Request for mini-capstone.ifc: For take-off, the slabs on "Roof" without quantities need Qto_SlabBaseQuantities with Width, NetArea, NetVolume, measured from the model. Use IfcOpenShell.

First a look at what the model holds.

```python
import ifcopenshell
import ifcopenshell.util.element
import ifcopenshell.util.unit

model = ifcopenshell.open("mini-capstone.ifc")
print(model.schema)
for unit_type in ("LENGTHUNIT", "AREAUNIT", "VOLUMEUNIT"):
    print(unit_type, ifcopenshell.util.unit.calculate_unit_scale(model, unit_type))
storey = next(s for s in model.by_type("IfcBuildingStorey") if s.Name == "Roof")
slabs = [e for e in ifcopenshell.util.element.get_decomposition(storey) if e.is_a("IfcSlab")]
for e in sorted(slabs, key=lambda e: e.id()):
    print(e.id(), e.is_a(), e.Name, list(ifcopenshell.util.element.get_psets(e, qtos_only=True)), sep=" | ")
```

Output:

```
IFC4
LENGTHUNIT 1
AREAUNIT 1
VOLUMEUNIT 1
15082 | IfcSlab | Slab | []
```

```python
import ifcopenshell
import ifcopenshell.api.pset
import ifcopenshell.geom
import ifcopenshell.util.element
import ifcopenshell.util.shape
import ifcopenshell.util.unit

model = ifcopenshell.open("mini-capstone.ifc")
unit_scale = ifcopenshell.util.unit.calculate_unit_scale(model)
area_scale = ifcopenshell.util.unit.calculate_unit_scale(model, "AREAUNIT")
volume_scale = ifcopenshell.util.unit.calculate_unit_scale(model, "VOLUMEUNIT")
settings = ifcopenshell.geom.settings()

storey = next(s for s in model.by_type("IfcBuildingStorey") if s.Name == "Roof")
slabs = [e for e in ifcopenshell.util.element.get_decomposition(storey) if e.is_a("IfcSlab")]

for e in sorted(slabs, key=lambda e: e.id()):
    if ifcopenshell.util.element.get_psets(e, qtos_only=True, should_inherit=False):
        continue
    # Geometry comes back in metres, in the element's own axes.
    shape = ifcopenshell.geom.create_shape(settings, e)
    values = {
        "Width": ifcopenshell.util.shape.get_z(shape.geometry) / unit_scale,
        "NetArea": ifcopenshell.util.shape.get_footprint_area(shape.geometry) / area_scale,
        "NetVolume": ifcopenshell.util.shape.get_volume(shape.geometry) / volume_scale,
    }
    qto = ifcopenshell.api.pset.add_qto(model, product=e, name="Qto_SlabBaseQuantities")
    ifcopenshell.api.pset.edit_qto(model, qto=qto, properties=values)
    print(e.id(), {k: round(v, 3) for k, v in values.items()})

model.write("mini-capstone_edited.ifc")
```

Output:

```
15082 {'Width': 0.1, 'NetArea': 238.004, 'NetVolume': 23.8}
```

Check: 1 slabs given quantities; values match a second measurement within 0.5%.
